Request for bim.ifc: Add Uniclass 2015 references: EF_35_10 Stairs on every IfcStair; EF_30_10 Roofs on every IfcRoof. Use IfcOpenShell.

First a look at what the model holds.

```python
import ifcopenshell

model = ifcopenshell.open("bim.ifc")
print(model.schema)
print("classifications:", [c.Name for c in model.by_type("IfcClassification")])
for ifc_class in ("IfcDoor", "IfcRoof", "IfcStair", "IfcWall", "IfcWindow"):
    print(ifc_class, len(model.by_type(ifc_class)))
```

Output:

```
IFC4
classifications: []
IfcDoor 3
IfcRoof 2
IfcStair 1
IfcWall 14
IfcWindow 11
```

```python
import ifcopenshell
import ifcopenshell.api.classification

model = ifcopenshell.open("bim.ifc")

system = ifcopenshell.api.classification.add_classification(model, classification="Uniclass 2015")

codes = {
    "IfcStair": ("EF_35_10", "Stairs"),
    "IfcRoof": ("EF_30_10", "Roofs"),
}
for ifc_class, (code, name) in codes.items():
    products = model.by_type(ifc_class)
    ifcopenshell.api.classification.add_reference(
        model, products=products, classification=system, identification=code, name=name
    )
    print(code, len(products))

model.write("bim_v2.ifc")
```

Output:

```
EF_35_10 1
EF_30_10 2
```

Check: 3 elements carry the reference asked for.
